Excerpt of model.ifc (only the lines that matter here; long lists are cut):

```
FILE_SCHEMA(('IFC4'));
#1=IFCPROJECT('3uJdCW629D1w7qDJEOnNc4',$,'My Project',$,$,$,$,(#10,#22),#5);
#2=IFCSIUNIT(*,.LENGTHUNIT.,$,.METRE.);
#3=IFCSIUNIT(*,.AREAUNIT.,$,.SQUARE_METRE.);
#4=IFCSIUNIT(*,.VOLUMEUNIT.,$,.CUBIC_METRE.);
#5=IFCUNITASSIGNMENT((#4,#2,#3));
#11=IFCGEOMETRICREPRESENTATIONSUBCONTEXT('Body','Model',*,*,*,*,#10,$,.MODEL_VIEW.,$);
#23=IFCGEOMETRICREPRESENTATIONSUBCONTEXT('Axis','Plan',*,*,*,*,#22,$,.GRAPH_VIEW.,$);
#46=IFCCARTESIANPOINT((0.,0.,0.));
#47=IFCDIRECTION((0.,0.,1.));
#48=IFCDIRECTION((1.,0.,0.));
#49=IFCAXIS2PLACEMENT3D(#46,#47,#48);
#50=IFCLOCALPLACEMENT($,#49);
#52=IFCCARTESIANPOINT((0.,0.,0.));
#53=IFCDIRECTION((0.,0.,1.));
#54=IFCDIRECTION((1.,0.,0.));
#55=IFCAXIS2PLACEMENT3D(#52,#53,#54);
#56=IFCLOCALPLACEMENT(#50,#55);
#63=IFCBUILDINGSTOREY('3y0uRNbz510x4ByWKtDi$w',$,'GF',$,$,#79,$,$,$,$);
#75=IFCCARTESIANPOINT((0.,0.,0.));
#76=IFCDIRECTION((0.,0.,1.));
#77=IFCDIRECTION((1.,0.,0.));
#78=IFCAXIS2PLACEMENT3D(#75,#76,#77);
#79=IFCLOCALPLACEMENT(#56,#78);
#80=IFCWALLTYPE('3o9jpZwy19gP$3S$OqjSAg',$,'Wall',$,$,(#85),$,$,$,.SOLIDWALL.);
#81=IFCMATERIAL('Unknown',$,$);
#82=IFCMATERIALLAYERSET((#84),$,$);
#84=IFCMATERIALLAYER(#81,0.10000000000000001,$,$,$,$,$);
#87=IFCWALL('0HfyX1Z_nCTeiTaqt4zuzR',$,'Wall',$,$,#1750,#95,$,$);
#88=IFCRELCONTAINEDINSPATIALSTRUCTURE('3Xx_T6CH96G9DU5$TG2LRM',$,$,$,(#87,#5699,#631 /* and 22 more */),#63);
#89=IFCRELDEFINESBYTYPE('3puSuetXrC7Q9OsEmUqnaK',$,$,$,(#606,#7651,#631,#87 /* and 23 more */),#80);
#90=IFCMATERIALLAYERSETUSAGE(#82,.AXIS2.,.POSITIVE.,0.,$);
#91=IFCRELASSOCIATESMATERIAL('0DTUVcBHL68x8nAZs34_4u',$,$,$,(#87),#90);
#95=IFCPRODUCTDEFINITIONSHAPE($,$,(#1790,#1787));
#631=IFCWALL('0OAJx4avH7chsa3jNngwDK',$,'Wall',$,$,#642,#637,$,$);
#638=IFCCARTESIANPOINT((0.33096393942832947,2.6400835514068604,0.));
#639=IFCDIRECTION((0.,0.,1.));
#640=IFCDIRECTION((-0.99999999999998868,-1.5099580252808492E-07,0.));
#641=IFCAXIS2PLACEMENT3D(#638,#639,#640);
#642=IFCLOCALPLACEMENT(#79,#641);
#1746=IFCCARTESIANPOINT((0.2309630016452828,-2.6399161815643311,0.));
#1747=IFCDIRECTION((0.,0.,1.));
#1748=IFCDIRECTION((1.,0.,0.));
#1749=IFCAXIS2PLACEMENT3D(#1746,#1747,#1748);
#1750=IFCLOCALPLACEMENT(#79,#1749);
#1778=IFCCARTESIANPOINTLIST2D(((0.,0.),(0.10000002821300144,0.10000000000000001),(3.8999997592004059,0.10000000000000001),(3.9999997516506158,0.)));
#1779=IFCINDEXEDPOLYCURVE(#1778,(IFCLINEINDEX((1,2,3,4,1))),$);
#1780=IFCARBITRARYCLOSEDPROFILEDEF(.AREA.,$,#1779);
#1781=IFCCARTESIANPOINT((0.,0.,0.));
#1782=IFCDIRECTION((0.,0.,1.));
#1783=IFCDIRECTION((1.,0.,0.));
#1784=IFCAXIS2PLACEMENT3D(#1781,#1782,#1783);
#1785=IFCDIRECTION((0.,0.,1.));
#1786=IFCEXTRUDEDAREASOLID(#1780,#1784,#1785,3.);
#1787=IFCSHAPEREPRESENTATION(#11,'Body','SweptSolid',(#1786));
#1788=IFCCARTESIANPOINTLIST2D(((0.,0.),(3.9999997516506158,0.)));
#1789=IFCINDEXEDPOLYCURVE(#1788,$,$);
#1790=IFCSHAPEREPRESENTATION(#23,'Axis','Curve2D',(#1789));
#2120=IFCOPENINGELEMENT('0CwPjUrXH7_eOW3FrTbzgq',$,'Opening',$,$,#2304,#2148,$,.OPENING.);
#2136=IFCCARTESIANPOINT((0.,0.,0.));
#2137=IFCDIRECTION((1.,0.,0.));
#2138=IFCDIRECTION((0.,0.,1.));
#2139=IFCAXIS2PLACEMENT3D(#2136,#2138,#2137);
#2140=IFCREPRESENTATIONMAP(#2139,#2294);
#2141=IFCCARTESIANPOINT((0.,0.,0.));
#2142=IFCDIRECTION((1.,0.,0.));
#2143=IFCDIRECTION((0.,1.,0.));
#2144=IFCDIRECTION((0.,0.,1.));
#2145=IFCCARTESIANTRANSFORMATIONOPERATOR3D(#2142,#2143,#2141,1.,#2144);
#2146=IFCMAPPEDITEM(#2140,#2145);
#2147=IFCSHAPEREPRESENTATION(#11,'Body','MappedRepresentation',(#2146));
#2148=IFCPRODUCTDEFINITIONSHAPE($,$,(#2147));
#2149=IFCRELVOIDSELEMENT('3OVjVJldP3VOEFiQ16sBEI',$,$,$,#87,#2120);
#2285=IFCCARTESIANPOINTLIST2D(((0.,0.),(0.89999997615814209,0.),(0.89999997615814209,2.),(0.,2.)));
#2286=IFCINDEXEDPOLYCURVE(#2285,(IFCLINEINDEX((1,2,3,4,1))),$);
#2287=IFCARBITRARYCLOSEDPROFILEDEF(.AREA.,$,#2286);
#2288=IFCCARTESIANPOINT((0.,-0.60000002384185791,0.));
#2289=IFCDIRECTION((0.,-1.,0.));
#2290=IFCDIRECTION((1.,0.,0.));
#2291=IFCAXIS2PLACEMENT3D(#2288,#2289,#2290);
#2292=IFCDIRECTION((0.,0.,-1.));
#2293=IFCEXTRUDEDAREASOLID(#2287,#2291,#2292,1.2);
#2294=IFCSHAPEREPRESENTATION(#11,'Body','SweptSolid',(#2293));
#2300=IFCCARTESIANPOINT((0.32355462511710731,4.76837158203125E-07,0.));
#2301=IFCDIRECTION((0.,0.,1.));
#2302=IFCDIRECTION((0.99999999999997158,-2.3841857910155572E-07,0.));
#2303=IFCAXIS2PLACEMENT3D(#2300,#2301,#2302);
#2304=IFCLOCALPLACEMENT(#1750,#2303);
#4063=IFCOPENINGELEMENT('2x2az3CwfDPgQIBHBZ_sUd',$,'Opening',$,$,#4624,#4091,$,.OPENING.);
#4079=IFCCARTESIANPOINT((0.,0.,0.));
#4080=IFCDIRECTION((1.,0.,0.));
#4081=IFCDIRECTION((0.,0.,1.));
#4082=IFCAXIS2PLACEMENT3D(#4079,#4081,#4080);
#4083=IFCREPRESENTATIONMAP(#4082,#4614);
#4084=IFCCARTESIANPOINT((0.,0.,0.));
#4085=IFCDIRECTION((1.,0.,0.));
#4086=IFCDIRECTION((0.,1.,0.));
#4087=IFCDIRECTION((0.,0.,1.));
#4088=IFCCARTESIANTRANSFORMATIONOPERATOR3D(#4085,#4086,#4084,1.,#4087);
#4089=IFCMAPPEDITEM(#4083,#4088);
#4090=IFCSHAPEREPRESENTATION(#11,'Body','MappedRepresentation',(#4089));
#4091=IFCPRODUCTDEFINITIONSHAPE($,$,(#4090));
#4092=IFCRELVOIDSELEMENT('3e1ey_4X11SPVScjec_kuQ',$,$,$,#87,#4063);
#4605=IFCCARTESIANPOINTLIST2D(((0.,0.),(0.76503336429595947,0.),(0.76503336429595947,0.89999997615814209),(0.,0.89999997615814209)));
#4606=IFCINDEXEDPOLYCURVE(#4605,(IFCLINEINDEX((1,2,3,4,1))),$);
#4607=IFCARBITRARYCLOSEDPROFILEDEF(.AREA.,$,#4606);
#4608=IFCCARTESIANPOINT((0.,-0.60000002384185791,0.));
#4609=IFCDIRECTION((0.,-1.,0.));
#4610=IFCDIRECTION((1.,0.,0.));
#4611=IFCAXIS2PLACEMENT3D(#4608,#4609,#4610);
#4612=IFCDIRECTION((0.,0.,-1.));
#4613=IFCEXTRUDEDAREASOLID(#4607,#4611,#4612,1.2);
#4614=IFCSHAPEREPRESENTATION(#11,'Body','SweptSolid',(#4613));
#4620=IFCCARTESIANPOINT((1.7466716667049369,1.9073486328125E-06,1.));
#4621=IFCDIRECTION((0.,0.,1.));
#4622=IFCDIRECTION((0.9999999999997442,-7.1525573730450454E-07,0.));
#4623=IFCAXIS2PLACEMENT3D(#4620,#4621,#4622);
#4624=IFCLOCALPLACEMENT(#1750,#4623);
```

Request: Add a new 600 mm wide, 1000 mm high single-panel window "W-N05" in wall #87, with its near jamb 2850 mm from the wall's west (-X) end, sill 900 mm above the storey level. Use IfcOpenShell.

```python
import numpy as np
import ifcopenshell
import ifcopenshell.api.feature
import ifcopenshell.api.geometry
import ifcopenshell.api.root
import ifcopenshell.api.spatial
import ifcopenshell.geom
import ifcopenshell.util.element
import ifcopenshell.util.placement
import ifcopenshell.util.representation
import ifcopenshell.util.shape
import ifcopenshell.util.unit

model = ifcopenshell.open("model.ifc")
unit_scale = ifcopenshell.util.unit.calculate_unit_scale(model)
settings = ifcopenshell.geom.settings()


def volume(element):
    """Net volume in cubic metres, openings subtracted."""
    shape = ifcopenshell.geom.create_shape(settings, element)
    return ifcopenshell.util.shape.get_volume(shape.geometry)


wall = model.by_id(87)
storey = ifcopenshell.util.element.get_container(wall, ifc_class="IfcBuildingStorey")
context = ifcopenshell.util.representation.get_context(model, "Model", "Body", "MODEL_VIEW")
before = volume(wall)

width, height, from_end, sill = 0.6, 1, 2.85, 0.9  # metres

# The wall runs along its own X axis, and the end named is its -X end.
wall_shape = ifcopenshell.geom.create_shape(settings, wall)
x, y, z = ifcopenshell.util.shape.get_vertices(wall_shape.geometry).T
start = x.min() + from_end
face, thickness = float(y.min()), float(y.max() - y.min())
wall_matrix = ifcopenshell.util.placement.get_local_placement(wall.ObjectPlacement)
level = ifcopenshell.util.placement.get_local_placement(storey.ObjectPlacement)[2, 3]


def in_wall(x, y):
    """Placement at x, y metres in the wall's axes, at sill height."""
    matrix = wall_matrix.copy()
    matrix[:, 3] = wall_matrix @ np.array([x / unit_scale, y / unit_scale, 0.0, 1.0])
    matrix[2, 3] = level + sill / unit_scale
    return matrix


# Opening: a box that overshoots both wall faces by 50 mm.
opening = ifcopenshell.api.root.create_entity(model, ifc_class="IfcOpeningElement", predefined_type="OPENING")
box = ifcopenshell.api.geometry.add_wall_representation(
    model, context=context, length=width, height=height, thickness=thickness + 0.1
)
ifcopenshell.api.geometry.assign_representation(model, product=opening, representation=box)
ifcopenshell.api.geometry.edit_object_placement(model, product=opening, matrix=in_wall(start, face - 0.05), is_si=False)
ifcopenshell.api.feature.add_feature(model, feature=opening, element=wall)

window = ifcopenshell.api.root.create_entity(model, ifc_class="IfcWindow", name="W-N05", predefined_type="WINDOW")
window.OverallWidth, window.OverallHeight = width / unit_scale, height / unit_scale
window.PartitioningType = "SINGLE_PANEL"
body = ifcopenshell.api.geometry.add_window_representation(
    model,
    context=context,
    overall_width=window.OverallWidth,
    overall_height=window.OverallHeight,
    partition_type="SINGLE_PANEL",
)
ifcopenshell.api.geometry.assign_representation(model, product=window, representation=body)
ifcopenshell.api.spatial.assign_container(model, products=[window], relating_structure=storey)
ifcopenshell.api.feature.add_filling(model, opening=opening, element=window)

# Centre the window in the wall's thickness.
ifcopenshell.api.geometry.edit_object_placement(model, product=window, matrix=in_wall(start, face), is_si=False)
window_shape = ifcopenshell.geom.create_shape(settings, window)
depth = ifcopenshell.util.shape.get_vertices(window_shape.geometry)[:, 1]
offset = face + thickness / 2 - (depth.min() + depth.max()) / 2
ifcopenshell.api.geometry.edit_object_placement(model, product=window, matrix=in_wall(start, offset), is_si=False)

after = volume(wall)

print(f"wall volume {before:.3f} -> {after:.3f} m3")

model.write("model_edited.ifc")
```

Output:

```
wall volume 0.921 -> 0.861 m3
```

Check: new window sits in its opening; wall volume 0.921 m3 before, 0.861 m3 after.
